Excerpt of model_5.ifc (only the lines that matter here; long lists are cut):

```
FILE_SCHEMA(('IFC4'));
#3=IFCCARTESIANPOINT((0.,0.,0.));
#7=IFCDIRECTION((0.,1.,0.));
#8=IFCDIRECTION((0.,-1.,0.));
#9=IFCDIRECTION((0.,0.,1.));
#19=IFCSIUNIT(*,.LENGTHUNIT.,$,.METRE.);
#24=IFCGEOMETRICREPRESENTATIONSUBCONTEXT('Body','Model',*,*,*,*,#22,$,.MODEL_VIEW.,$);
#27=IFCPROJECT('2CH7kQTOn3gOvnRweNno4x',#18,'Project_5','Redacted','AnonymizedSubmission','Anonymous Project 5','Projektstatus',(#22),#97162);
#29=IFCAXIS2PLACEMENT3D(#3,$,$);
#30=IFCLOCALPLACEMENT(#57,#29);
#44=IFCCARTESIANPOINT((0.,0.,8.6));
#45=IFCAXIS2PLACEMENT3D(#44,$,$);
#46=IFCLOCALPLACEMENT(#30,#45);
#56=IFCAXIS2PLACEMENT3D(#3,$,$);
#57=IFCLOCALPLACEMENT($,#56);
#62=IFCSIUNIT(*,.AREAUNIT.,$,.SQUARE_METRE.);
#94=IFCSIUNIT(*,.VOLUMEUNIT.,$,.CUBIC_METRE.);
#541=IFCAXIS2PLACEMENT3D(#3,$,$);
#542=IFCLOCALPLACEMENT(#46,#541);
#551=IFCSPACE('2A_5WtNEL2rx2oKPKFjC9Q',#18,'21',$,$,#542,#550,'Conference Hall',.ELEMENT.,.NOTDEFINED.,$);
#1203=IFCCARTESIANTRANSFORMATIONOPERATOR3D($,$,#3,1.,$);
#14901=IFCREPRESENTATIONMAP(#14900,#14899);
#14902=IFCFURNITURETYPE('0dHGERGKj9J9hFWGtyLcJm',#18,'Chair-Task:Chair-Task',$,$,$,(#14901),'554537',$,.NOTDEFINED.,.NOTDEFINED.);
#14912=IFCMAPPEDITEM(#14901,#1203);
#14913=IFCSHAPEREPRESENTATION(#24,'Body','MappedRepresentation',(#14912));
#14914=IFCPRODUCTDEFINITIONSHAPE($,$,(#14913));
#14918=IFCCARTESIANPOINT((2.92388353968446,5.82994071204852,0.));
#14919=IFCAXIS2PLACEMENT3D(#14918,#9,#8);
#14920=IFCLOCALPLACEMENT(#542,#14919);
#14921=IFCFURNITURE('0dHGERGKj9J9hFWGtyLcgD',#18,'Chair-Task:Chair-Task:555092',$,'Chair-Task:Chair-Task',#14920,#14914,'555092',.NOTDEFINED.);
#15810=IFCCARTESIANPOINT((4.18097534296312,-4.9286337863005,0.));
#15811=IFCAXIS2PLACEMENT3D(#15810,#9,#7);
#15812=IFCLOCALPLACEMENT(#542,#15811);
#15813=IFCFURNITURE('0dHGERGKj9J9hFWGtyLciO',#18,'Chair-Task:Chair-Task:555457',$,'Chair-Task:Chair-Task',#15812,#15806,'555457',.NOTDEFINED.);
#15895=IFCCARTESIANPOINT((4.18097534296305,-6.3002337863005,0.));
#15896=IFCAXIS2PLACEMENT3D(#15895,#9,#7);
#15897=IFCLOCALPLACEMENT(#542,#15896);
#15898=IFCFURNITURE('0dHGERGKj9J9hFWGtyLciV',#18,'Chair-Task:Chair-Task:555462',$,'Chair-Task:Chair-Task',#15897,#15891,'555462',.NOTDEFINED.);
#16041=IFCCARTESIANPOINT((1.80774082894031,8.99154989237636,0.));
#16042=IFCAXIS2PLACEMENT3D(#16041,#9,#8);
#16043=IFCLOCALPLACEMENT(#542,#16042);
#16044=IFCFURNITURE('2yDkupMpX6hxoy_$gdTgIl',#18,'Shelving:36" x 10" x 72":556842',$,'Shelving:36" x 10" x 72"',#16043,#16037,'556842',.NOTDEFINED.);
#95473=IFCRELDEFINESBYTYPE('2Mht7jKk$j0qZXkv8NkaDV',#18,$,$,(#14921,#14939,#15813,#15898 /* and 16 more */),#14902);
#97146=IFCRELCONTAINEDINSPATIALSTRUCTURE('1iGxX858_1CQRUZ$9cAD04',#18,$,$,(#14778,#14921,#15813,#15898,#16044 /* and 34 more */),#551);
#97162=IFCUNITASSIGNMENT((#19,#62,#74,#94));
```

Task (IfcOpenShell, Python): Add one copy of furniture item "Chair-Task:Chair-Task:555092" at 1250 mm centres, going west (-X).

```python
import numpy as np
import ifcopenshell
import ifcopenshell.api.geometry
import ifcopenshell.api.root
import ifcopenshell.util.element
import ifcopenshell.util.placement
import ifcopenshell.util.unit

model = ifcopenshell.open("model_5.ifc")
unit_scale = ifcopenshell.util.unit.calculate_unit_scale(model)


def reuse_history(source, copy):
    """copy_class also copies each property set's owner history, people and application; keep the originals."""
    for rel in copy.IsDefinedBy:
        if rel.is_a("IfcRelDefinesByProperties") and (history := rel.RelatingPropertyDefinition.OwnerHistory):
            rel.RelatingPropertyDefinition.OwnerHistory = source.OwnerHistory
            ifcopenshell.util.element.remove_deep2(model, history)


source = model.by_guid("0dHGERGKj9J9hFWGtyLcgD")
base = ifcopenshell.util.placement.get_local_placement(source.ObjectPlacement)
step = np.array([-1.0, 0.0, 0.0]) * 1.25 / unit_scale

for i in range(1, 2):
    copy = ifcopenshell.api.root.copy_class(model, product=source)
    copy.Representation = ifcopenshell.util.element.copy_deep(
        model, source.Representation, exclude=["IfcGeometricRepresentationContext", "IfcRepresentationMap"]
    )
    copy.Name = "Chair-Task:Chair-Task"
    copy.Tag = None
    reuse_history(source, copy)
    matrix = base.copy()
    matrix[:3, 3] += i * step
    print("added at", matrix[:3, 3].round(3) + 0.0)
    ifcopenshell.api.geometry.edit_object_placement(model, product=copy, matrix=matrix, is_si=False)

model.write("model_5_edited.ifc")
```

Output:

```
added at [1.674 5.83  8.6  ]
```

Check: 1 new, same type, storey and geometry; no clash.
